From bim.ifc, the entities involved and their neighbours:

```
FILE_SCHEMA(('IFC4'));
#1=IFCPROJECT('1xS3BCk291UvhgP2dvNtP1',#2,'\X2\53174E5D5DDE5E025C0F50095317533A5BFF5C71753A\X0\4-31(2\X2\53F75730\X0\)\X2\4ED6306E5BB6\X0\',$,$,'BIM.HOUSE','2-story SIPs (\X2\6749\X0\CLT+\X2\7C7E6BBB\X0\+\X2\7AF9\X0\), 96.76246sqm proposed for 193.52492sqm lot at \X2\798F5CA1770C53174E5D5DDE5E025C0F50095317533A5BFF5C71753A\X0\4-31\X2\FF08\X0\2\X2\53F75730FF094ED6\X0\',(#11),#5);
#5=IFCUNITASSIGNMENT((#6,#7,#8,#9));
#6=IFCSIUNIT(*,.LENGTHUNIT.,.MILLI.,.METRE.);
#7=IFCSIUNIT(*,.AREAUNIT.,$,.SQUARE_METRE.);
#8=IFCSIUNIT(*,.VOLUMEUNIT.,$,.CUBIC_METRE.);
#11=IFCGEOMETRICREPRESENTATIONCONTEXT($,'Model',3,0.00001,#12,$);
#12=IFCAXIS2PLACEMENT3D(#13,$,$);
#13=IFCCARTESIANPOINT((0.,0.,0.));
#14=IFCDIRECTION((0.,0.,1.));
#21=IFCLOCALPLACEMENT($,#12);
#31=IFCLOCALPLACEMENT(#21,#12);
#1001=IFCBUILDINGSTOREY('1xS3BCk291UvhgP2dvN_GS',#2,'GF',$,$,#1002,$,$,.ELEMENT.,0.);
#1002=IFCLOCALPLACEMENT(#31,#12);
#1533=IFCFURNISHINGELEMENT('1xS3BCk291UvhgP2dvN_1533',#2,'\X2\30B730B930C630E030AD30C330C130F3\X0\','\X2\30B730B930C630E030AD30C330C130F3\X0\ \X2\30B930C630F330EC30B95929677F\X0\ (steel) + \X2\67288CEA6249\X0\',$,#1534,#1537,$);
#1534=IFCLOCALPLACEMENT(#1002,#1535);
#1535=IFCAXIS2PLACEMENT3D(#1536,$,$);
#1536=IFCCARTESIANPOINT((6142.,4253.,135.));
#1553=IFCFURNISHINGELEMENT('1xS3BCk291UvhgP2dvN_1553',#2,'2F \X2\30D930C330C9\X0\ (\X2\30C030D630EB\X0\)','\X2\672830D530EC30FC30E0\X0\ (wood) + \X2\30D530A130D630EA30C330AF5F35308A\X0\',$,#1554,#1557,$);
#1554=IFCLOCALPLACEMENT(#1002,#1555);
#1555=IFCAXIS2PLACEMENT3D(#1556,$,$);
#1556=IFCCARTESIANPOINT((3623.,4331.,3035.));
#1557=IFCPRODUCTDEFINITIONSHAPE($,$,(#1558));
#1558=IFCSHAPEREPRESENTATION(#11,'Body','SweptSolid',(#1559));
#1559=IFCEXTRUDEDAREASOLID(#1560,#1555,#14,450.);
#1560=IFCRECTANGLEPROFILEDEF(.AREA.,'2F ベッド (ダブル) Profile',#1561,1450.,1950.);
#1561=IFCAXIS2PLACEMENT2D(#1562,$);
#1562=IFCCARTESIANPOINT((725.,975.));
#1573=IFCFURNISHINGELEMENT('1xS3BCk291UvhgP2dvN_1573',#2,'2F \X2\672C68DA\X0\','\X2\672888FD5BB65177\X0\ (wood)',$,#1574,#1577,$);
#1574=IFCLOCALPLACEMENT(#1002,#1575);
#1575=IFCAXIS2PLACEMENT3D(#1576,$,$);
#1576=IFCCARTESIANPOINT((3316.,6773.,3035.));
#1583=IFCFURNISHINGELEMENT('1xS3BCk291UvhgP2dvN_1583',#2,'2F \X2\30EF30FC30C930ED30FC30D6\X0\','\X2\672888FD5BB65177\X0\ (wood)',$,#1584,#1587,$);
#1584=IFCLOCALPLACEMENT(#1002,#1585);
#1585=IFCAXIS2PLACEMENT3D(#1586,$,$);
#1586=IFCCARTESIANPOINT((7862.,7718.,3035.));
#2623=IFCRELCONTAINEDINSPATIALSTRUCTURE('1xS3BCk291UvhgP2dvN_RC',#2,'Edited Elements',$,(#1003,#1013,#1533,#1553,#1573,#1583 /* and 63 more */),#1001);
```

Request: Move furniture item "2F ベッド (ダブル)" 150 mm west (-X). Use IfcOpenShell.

```python
import ifcopenshell
import ifcopenshell.api.geometry
import ifcopenshell.util.placement

model = ifcopenshell.open("bim.ifc")

item = model.by_id(1553)
matrix = ifcopenshell.util.placement.get_local_placement(item.ObjectPlacement)
matrix[0, 3] -= 150.0
ifcopenshell.api.geometry.edit_object_placement(model, product=item, matrix=matrix, is_si=False)

print(ifcopenshell.util.placement.get_local_placement(item.ObjectPlacement).round(3) + 0.0)

model.write("bim_updated.ifc")
```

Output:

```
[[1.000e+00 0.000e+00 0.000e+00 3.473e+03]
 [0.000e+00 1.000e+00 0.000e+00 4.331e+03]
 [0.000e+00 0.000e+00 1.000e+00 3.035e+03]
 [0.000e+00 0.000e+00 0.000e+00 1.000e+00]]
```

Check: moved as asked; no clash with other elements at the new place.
